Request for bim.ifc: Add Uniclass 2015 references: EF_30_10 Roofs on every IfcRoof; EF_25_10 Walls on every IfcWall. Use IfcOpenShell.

First a look at what the model holds.

```python
import ifcopenshell

model = ifcopenshell.open("bim.ifc")
print(model.schema)
print("classifications:", [c.Name for c in model.by_type("IfcClassification")])
for ifc_class in ("IfcDoor", "IfcRoof", "IfcStair", "IfcWall", "IfcWindow"):
    print(ifc_class, len(model.by_type(ifc_class)))
```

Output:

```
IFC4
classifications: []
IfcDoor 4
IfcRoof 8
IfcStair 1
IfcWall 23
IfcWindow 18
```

```python
import ifcopenshell
import ifcopenshell.api.classification

model = ifcopenshell.open("bim.ifc")

system = ifcopenshell.api.classification.add_classification(model, classification="Uniclass 2015")

codes = {
    "IfcRoof": ("EF_30_10", "Roofs"),
    "IfcWall": ("EF_25_10", "Walls"),
}
for ifc_class, (code, name) in codes.items():
    products = model.by_type(ifc_class)
    ifcopenshell.api.classification.add_reference(
        model, products=products, classification=system, identification=code, name=name
    )
    print(code, len(products))

model.write("bim_edited.ifc")
```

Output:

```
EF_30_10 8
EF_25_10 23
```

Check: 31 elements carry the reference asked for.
